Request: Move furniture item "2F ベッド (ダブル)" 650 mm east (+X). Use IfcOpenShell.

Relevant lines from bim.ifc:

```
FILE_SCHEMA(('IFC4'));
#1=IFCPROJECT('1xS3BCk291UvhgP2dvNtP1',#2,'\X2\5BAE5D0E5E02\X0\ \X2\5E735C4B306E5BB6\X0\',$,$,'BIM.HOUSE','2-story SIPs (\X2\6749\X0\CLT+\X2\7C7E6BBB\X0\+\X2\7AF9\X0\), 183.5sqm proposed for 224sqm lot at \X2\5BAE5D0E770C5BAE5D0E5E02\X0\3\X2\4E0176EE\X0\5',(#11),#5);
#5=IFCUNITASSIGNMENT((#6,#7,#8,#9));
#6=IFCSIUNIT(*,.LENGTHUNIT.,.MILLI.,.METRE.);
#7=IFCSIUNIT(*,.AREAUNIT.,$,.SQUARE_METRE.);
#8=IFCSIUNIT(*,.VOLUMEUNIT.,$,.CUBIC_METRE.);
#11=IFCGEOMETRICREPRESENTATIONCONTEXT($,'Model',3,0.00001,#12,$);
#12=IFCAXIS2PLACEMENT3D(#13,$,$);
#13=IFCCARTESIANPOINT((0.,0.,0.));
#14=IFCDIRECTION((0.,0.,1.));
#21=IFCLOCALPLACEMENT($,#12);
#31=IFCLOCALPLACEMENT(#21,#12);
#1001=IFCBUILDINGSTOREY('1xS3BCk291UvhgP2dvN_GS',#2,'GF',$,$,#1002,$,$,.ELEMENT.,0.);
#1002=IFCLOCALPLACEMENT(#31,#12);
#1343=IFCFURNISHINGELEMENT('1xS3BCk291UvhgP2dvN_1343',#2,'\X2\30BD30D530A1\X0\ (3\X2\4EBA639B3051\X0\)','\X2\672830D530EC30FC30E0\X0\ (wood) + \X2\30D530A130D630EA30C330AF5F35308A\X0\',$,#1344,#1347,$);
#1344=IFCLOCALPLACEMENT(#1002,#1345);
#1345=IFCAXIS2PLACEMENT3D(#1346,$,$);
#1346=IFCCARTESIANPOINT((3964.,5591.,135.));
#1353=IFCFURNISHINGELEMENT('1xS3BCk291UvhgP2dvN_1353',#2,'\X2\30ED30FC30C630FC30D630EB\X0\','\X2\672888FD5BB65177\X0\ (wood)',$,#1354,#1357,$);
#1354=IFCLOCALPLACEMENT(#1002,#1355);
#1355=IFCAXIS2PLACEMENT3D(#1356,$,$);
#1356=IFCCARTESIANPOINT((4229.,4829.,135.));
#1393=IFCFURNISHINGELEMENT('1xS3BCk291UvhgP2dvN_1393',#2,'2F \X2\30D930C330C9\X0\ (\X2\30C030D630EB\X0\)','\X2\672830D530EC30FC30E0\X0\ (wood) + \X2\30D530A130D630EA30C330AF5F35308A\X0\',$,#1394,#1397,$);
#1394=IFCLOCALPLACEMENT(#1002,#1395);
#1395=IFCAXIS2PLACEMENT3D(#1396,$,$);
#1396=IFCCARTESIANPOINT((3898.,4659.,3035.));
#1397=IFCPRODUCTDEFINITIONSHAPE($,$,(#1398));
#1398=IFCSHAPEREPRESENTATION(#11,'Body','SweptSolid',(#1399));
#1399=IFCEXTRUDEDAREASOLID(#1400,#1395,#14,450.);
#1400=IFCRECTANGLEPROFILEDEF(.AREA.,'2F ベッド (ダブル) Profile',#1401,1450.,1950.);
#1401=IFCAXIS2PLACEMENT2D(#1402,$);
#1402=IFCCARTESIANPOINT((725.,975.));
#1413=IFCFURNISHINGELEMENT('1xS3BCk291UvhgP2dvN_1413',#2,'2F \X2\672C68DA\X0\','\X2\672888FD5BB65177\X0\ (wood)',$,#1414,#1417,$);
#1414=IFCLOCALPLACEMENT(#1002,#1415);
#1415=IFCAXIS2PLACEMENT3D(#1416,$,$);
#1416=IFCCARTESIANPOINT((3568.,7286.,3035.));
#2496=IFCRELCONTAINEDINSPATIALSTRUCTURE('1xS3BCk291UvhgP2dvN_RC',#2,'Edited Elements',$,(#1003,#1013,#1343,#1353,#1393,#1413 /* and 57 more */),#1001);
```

```python
import ifcopenshell
import ifcopenshell.api.geometry
import ifcopenshell.util.placement

model = ifcopenshell.open("bim.ifc")

item = model.by_id(1393)
matrix = ifcopenshell.util.placement.get_local_placement(item.ObjectPlacement)
matrix[0, 3] += 650.0
ifcopenshell.api.geometry.edit_object_placement(model, product=item, matrix=matrix, is_si=False)

print(ifcopenshell.util.placement.get_local_placement(item.ObjectPlacement).round(3) + 0.0)

model.write("bim_edited.ifc")
```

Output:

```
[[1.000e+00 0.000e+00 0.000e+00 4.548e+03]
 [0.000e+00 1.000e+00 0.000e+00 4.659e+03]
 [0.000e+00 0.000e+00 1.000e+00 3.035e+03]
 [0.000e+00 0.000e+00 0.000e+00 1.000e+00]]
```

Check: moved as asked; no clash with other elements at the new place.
